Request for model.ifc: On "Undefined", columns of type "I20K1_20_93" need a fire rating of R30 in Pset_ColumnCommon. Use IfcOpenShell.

First a look at what the model holds.

```python
import ifcopenshell
import ifcopenshell.util.element

model = ifcopenshell.open("model.ifc")
print(model.schema)
storey = next(s for s in model.by_type("IfcBuildingStorey") if s.Name == "Undefined")
columns = [e for e in ifcopenshell.util.element.get_decomposition(storey) if e.is_a("IfcColumn")]
seen = {}
for e in columns:
    element_type = ifcopenshell.util.element.get_type(e)
    key = (element_type.Name if element_type != e and element_type else None, ifcopenshell.util.element.get_pset(e, "Pset_ColumnCommon", "FireRating"))
    seen[key] = seen.get(key, 0) + 1
for (name, value), count in sorted(seen.items(), key=str):
    print(count, "x", name, "|", value)
```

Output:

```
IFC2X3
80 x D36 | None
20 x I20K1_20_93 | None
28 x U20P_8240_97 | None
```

```python
import ifcopenshell
import ifcopenshell.api.pset
import ifcopenshell.util.element

model = ifcopenshell.open("model.ifc")

storey = next(s for s in model.by_type("IfcBuildingStorey") if s.Name == "Undefined")
columns = [e for e in ifcopenshell.util.element.get_decomposition(storey) if e.is_a("IfcColumn")]

count = 0
for e in columns:
    element_type = ifcopenshell.util.element.get_type(e)
    if element_type in (None, e) or element_type.Name != "I20K1_20_93":
        continue
    found = ifcopenshell.util.element.get_pset(e, "Pset_ColumnCommon", should_inherit=False)
    if found:
        pset = model.by_id(found["id"])
        if len(ifcopenshell.util.element.get_elements_by_pset(pset)) > 1:
            pset = ifcopenshell.api.pset.unshare_pset(model, products=[e], pset=pset)[0]
    else:
        pset = ifcopenshell.api.pset.add_pset(model, product=e, name="Pset_ColumnCommon")
    ifcopenshell.api.pset.edit_pset(model, pset=pset, properties={"FireRating": "R30"})
    count += 1

print(count, "columns updated")

model.write("model-out.ifc")
```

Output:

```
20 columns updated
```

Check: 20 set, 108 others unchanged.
